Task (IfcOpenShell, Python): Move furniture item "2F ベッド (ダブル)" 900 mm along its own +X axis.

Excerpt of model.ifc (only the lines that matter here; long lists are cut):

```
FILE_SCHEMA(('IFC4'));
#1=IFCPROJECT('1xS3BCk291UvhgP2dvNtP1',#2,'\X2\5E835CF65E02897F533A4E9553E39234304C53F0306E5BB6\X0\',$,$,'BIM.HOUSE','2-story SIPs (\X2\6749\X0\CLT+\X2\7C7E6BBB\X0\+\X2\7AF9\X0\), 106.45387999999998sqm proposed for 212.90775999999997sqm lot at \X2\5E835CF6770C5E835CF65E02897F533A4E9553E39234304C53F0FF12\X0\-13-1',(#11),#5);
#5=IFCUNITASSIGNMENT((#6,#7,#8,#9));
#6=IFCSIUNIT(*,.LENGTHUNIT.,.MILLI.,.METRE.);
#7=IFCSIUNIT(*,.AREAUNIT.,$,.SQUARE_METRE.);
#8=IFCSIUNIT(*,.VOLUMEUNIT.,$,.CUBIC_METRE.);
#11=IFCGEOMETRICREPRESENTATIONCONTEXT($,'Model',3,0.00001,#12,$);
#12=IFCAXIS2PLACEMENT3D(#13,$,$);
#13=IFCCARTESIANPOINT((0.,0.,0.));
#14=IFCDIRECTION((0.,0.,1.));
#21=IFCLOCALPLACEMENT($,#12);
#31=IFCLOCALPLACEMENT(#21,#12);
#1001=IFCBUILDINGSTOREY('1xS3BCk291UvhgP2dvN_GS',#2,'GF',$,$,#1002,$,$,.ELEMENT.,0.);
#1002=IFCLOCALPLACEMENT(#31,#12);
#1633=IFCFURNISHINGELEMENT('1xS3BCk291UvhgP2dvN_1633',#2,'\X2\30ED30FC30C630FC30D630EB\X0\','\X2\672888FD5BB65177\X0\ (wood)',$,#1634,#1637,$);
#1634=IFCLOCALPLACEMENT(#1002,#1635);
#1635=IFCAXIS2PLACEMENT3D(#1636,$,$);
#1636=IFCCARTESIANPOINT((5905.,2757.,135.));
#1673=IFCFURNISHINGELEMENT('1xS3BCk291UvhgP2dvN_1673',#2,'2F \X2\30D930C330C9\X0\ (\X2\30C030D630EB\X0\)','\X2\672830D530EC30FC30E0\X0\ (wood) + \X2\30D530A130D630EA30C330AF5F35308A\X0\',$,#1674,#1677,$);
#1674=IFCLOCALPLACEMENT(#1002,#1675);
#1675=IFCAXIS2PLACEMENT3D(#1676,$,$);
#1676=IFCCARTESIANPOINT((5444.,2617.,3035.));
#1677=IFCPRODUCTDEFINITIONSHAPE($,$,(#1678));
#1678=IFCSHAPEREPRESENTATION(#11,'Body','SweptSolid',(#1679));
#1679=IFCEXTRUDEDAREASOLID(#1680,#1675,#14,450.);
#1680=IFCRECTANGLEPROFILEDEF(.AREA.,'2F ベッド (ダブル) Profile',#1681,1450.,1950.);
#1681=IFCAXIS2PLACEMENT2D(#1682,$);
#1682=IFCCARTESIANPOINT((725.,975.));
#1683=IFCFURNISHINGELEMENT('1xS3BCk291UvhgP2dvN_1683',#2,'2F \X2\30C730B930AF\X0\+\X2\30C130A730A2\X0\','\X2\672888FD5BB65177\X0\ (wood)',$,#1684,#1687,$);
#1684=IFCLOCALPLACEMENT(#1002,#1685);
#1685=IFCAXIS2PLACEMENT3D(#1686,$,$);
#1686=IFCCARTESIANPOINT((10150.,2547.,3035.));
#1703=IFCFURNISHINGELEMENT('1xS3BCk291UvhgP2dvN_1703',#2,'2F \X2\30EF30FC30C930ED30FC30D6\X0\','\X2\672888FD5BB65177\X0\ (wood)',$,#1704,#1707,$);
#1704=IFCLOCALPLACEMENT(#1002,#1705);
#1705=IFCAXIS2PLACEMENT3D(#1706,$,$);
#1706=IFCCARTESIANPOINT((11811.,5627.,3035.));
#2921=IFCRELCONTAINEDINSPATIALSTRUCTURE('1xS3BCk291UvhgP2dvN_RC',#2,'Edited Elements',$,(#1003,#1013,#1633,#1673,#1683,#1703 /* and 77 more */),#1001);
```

```python
import ifcopenshell
import ifcopenshell.api.geometry
import ifcopenshell.util.placement
import ifcopenshell.util.unit

model = ifcopenshell.open("model.ifc")
unit_scale = ifcopenshell.util.unit.calculate_unit_scale(model)

item = model.by_guid("1xS3BCk291UvhgP2dvN_1673")
matrix = ifcopenshell.util.placement.get_local_placement(item.ObjectPlacement)
matrix[:3, 3] += matrix[:3, 0] * 0.9 / unit_scale
ifcopenshell.api.geometry.edit_object_placement(model, product=item, matrix=matrix, is_si=False)

print(ifcopenshell.util.placement.get_local_placement(item.ObjectPlacement).round(3) + 0.0)

model.write("model_updated.ifc")
```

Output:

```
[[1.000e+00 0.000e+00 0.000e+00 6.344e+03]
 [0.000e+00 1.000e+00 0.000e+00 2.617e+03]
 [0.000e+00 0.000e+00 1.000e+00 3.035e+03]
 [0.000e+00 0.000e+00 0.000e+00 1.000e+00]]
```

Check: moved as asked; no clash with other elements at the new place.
